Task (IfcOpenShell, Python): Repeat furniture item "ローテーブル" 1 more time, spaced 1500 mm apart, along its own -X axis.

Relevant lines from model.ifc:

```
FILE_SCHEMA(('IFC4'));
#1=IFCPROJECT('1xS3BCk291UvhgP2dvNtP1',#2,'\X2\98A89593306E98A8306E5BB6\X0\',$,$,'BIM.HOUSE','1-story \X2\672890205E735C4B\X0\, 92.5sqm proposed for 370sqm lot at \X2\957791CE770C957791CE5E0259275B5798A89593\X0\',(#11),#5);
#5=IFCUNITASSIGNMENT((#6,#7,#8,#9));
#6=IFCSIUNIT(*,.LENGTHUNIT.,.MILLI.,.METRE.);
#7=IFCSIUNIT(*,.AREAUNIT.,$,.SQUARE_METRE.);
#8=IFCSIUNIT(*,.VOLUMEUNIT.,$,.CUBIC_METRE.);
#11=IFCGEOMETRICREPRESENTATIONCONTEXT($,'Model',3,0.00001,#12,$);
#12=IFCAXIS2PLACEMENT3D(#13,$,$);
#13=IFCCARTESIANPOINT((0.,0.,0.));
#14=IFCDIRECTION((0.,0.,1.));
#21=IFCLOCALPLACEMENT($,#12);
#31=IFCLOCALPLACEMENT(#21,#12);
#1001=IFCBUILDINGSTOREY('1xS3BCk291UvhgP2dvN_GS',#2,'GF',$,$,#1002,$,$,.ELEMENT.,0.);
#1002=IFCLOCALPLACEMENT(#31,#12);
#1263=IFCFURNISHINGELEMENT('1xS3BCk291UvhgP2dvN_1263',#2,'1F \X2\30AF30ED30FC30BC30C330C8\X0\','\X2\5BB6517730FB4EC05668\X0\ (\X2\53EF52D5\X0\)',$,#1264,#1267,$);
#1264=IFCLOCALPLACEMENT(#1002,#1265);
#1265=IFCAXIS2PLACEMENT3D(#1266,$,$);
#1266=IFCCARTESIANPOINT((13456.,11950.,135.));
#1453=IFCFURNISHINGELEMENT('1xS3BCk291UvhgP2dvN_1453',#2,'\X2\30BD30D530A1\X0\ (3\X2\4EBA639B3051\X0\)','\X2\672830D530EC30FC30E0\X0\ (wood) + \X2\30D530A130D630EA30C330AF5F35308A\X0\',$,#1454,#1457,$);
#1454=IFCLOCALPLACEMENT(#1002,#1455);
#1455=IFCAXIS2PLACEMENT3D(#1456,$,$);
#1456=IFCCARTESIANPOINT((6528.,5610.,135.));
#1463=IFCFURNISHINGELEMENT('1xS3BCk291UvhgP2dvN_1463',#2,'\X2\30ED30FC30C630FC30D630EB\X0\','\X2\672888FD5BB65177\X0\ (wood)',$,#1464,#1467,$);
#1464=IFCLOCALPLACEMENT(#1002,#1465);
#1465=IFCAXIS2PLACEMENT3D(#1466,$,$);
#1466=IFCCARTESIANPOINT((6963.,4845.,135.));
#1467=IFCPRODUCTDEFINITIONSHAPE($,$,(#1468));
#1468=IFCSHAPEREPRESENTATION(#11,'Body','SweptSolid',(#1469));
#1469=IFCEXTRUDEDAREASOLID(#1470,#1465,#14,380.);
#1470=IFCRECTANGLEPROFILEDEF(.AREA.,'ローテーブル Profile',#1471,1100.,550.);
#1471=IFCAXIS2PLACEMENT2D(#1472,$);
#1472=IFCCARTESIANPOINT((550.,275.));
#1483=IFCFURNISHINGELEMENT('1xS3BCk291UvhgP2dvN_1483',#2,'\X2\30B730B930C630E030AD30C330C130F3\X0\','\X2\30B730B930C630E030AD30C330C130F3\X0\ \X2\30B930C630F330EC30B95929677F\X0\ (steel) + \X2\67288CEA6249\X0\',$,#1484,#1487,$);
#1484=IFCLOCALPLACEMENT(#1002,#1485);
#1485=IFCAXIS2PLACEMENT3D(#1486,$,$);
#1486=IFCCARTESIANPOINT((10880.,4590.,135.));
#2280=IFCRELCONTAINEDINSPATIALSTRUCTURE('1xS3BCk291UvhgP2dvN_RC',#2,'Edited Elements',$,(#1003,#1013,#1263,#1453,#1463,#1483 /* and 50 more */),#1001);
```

```python
import ifcopenshell
import ifcopenshell.api.geometry
import ifcopenshell.api.root
import ifcopenshell.util.element
import ifcopenshell.util.placement
import ifcopenshell.util.unit

model = ifcopenshell.open("model.ifc")
unit_scale = ifcopenshell.util.unit.calculate_unit_scale(model)


def reuse_history(source, copy):
    """copy_class also copies each property set's owner history, people and application; keep the originals."""
    for rel in copy.IsDefinedBy:
        if rel.is_a("IfcRelDefinesByProperties") and (history := rel.RelatingPropertyDefinition.OwnerHistory):
            rel.RelatingPropertyDefinition.OwnerHistory = source.OwnerHistory
            ifcopenshell.util.element.remove_deep2(model, history)


source = model.by_id(1463)
base = ifcopenshell.util.placement.get_local_placement(source.ObjectPlacement)
step = -base[:3, 0] * 1.5 / unit_scale

for i in range(1, 2):
    copy = ifcopenshell.api.root.copy_class(model, product=source)
    copy.Representation = ifcopenshell.util.element.copy_deep(
        model, source.Representation, exclude=["IfcGeometricRepresentationContext", "IfcRepresentationMap"]
    )
    reuse_history(source, copy)
    matrix = base.copy()
    matrix[:3, 3] += i * step
    print("added at", matrix[:3, 3].round(3) + 0.0)
    ifcopenshell.api.geometry.edit_object_placement(model, product=copy, matrix=matrix, is_si=False)

model.write("model-out.ifc")
```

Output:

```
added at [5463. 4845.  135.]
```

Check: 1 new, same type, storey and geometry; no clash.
